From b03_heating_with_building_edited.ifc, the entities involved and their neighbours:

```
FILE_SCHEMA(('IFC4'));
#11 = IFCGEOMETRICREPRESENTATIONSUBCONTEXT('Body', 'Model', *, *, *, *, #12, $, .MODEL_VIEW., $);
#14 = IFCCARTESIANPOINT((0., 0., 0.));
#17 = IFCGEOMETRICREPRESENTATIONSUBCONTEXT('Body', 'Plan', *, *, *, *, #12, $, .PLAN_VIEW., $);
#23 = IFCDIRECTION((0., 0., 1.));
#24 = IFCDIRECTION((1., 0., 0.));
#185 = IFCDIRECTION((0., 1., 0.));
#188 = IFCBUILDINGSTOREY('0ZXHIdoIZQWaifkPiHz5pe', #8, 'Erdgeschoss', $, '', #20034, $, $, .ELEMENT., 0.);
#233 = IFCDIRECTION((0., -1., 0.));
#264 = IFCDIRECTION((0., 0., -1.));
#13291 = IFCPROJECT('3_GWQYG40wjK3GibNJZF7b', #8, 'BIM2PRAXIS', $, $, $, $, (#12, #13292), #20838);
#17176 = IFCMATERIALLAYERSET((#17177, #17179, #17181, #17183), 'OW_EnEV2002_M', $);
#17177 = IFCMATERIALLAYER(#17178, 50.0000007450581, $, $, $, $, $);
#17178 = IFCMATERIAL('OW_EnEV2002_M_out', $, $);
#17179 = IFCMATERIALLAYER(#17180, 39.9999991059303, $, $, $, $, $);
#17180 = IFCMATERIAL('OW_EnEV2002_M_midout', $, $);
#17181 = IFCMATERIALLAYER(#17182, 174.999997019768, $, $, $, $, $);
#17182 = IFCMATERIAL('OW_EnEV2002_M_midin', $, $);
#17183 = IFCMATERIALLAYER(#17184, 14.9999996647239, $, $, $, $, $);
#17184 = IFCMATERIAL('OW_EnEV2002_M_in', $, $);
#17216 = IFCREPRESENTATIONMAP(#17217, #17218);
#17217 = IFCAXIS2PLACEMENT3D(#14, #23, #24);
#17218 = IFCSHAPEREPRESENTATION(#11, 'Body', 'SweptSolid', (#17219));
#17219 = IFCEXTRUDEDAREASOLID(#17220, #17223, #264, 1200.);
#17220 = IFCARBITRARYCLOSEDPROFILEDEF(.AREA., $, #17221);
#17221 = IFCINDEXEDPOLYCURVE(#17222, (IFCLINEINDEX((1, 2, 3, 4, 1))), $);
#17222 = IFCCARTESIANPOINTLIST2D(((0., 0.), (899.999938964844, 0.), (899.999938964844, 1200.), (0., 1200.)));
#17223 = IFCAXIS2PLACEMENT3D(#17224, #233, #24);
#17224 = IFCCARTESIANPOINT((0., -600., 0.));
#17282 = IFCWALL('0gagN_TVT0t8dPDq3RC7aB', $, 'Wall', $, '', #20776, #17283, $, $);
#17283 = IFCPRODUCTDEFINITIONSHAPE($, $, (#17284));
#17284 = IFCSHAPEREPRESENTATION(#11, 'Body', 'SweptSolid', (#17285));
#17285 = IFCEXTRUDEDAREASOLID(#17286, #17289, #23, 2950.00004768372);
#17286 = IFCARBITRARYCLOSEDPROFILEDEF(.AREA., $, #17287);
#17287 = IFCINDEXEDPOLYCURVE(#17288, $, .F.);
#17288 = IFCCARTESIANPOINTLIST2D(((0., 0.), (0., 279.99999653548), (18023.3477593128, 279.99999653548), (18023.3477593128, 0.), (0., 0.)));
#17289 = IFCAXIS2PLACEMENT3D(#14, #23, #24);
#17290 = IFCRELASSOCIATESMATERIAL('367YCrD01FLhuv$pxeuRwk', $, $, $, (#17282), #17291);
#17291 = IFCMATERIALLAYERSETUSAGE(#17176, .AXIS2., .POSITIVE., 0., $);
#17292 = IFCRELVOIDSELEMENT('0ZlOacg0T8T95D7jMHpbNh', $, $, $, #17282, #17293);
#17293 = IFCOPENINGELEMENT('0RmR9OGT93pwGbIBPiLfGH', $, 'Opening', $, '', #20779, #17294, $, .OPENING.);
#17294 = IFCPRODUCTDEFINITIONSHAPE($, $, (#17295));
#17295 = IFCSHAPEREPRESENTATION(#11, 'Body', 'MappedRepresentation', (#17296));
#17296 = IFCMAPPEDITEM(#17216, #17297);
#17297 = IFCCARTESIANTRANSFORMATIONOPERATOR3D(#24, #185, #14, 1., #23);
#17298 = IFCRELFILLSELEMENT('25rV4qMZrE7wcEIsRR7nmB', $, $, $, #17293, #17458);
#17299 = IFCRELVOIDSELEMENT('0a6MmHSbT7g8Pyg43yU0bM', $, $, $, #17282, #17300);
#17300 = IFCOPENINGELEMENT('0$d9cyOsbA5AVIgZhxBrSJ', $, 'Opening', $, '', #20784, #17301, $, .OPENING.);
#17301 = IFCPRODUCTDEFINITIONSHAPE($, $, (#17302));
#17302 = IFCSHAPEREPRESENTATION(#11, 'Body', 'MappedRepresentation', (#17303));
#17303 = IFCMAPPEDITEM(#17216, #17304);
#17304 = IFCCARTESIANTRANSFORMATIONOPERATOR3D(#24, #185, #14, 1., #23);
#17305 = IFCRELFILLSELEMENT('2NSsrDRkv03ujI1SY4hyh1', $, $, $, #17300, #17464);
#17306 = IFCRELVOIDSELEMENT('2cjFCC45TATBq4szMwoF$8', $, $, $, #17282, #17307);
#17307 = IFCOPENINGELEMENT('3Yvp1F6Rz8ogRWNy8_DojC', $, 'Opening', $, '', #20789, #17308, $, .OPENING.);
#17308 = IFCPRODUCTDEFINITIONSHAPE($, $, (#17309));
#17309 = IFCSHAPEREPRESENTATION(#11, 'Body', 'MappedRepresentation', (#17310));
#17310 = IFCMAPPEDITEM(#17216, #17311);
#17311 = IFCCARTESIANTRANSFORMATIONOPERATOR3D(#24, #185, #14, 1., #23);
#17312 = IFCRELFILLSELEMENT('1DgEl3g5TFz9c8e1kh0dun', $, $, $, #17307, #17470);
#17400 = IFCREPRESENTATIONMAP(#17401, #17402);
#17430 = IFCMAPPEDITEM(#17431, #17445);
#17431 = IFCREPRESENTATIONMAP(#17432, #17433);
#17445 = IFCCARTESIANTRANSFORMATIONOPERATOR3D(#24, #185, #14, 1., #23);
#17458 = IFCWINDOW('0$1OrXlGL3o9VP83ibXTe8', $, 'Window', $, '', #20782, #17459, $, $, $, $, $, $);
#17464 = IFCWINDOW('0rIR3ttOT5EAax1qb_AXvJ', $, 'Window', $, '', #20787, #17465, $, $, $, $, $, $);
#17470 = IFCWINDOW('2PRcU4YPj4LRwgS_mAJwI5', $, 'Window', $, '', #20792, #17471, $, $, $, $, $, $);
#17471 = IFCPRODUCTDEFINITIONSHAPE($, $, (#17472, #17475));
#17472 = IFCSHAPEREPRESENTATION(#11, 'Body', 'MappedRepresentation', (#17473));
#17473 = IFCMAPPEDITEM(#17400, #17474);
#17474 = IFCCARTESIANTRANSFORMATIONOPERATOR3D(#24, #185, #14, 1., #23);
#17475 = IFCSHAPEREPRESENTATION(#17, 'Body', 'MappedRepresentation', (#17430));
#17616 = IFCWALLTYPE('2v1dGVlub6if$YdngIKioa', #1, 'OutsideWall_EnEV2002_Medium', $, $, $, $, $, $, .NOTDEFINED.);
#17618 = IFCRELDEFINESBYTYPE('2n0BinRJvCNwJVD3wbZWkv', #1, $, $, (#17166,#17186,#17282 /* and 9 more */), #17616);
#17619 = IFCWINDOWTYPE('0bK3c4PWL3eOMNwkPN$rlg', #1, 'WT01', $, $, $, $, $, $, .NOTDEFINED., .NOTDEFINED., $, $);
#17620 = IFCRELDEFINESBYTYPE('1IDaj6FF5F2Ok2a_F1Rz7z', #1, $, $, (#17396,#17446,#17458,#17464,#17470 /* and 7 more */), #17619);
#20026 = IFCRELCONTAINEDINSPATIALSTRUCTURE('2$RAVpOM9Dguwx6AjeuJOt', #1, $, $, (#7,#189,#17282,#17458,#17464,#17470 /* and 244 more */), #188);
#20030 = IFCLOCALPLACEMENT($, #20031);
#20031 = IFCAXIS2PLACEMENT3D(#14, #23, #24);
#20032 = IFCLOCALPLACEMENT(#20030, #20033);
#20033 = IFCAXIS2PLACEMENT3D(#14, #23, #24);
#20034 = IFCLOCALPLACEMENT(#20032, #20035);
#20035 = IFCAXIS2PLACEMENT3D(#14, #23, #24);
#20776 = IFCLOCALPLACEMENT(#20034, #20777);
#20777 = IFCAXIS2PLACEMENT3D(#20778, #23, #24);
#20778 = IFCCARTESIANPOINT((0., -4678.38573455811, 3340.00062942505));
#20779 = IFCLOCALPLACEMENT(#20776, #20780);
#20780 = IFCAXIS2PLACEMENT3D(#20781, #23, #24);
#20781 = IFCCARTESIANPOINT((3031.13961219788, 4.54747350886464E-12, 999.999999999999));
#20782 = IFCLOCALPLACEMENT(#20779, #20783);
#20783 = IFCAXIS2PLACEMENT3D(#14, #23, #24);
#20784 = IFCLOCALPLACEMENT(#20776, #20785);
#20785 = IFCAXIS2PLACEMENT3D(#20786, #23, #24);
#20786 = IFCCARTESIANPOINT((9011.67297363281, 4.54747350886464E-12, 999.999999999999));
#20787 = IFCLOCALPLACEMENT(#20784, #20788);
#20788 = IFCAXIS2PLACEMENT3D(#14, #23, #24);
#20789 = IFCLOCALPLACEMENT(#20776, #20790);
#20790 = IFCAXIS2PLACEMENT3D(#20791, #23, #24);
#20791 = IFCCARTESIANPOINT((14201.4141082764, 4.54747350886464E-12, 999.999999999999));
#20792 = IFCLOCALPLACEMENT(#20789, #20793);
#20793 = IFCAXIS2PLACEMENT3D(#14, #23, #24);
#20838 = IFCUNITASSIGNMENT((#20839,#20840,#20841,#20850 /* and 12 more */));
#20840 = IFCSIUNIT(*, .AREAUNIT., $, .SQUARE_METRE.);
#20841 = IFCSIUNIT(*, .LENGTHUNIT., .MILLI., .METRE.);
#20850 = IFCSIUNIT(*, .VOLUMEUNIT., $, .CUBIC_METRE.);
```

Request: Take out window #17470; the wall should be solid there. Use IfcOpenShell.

```python
import ifcopenshell
import ifcopenshell.api.feature
import ifcopenshell.api.root
import ifcopenshell.geom
import ifcopenshell.util.shape

model = ifcopenshell.open("b03_heating_with_building_edited.ifc")
settings = ifcopenshell.geom.settings()


def volume(element):
    """Net volume in cubic metres, openings subtracted."""
    shape = ifcopenshell.geom.create_shape(settings, element)
    return ifcopenshell.util.shape.get_volume(shape.geometry)


window = model.by_guid("2PRcU4YPj4LRwgS_mAJwI5")
opening = window.FillsVoids[0].RelatingOpeningElement
wall = opening.VoidsElements[0].RelatingBuildingElement
before = volume(wall)

ifcopenshell.api.root.remove_product(model, product=window)
ifcopenshell.api.feature.remove_feature(model, feature=opening)

after = volume(wall)

print(f"wall volume {before:.3f} -> {after:.3f} m3")

model.write("b03_heating_with_building_edited_v2.ifc")
```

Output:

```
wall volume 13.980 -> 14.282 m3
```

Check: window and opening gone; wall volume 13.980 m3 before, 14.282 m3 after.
